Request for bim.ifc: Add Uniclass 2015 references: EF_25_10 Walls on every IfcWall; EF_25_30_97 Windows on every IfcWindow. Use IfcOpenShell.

First a look at what the model holds.

```python
import ifcopenshell

model = ifcopenshell.open("bim.ifc")
print(model.schema)
print("classifications:", [c.Name for c in model.by_type("IfcClassification")])
for ifc_class in ("IfcDoor", "IfcRoof", "IfcStair", "IfcWall", "IfcWindow"):
    print(ifc_class, len(model.by_type(ifc_class)))
```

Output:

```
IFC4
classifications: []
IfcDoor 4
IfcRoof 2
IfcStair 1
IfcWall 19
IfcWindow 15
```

```python
import ifcopenshell
import ifcopenshell.api.classification

model = ifcopenshell.open("bim.ifc")

system = ifcopenshell.api.classification.add_classification(model, classification="Uniclass 2015")

codes = {
    "IfcWall": ("EF_25_10", "Walls"),
    "IfcWindow": ("EF_25_30_97", "Windows"),
}
for ifc_class, (code, name) in codes.items():
    products = model.by_type(ifc_class)
    ifcopenshell.api.classification.add_reference(
        model, products=products, classification=system, identification=code, name=name
    )
    print(code, len(products))

model.write("bim-out.ifc")
```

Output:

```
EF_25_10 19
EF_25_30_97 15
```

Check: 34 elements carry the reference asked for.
